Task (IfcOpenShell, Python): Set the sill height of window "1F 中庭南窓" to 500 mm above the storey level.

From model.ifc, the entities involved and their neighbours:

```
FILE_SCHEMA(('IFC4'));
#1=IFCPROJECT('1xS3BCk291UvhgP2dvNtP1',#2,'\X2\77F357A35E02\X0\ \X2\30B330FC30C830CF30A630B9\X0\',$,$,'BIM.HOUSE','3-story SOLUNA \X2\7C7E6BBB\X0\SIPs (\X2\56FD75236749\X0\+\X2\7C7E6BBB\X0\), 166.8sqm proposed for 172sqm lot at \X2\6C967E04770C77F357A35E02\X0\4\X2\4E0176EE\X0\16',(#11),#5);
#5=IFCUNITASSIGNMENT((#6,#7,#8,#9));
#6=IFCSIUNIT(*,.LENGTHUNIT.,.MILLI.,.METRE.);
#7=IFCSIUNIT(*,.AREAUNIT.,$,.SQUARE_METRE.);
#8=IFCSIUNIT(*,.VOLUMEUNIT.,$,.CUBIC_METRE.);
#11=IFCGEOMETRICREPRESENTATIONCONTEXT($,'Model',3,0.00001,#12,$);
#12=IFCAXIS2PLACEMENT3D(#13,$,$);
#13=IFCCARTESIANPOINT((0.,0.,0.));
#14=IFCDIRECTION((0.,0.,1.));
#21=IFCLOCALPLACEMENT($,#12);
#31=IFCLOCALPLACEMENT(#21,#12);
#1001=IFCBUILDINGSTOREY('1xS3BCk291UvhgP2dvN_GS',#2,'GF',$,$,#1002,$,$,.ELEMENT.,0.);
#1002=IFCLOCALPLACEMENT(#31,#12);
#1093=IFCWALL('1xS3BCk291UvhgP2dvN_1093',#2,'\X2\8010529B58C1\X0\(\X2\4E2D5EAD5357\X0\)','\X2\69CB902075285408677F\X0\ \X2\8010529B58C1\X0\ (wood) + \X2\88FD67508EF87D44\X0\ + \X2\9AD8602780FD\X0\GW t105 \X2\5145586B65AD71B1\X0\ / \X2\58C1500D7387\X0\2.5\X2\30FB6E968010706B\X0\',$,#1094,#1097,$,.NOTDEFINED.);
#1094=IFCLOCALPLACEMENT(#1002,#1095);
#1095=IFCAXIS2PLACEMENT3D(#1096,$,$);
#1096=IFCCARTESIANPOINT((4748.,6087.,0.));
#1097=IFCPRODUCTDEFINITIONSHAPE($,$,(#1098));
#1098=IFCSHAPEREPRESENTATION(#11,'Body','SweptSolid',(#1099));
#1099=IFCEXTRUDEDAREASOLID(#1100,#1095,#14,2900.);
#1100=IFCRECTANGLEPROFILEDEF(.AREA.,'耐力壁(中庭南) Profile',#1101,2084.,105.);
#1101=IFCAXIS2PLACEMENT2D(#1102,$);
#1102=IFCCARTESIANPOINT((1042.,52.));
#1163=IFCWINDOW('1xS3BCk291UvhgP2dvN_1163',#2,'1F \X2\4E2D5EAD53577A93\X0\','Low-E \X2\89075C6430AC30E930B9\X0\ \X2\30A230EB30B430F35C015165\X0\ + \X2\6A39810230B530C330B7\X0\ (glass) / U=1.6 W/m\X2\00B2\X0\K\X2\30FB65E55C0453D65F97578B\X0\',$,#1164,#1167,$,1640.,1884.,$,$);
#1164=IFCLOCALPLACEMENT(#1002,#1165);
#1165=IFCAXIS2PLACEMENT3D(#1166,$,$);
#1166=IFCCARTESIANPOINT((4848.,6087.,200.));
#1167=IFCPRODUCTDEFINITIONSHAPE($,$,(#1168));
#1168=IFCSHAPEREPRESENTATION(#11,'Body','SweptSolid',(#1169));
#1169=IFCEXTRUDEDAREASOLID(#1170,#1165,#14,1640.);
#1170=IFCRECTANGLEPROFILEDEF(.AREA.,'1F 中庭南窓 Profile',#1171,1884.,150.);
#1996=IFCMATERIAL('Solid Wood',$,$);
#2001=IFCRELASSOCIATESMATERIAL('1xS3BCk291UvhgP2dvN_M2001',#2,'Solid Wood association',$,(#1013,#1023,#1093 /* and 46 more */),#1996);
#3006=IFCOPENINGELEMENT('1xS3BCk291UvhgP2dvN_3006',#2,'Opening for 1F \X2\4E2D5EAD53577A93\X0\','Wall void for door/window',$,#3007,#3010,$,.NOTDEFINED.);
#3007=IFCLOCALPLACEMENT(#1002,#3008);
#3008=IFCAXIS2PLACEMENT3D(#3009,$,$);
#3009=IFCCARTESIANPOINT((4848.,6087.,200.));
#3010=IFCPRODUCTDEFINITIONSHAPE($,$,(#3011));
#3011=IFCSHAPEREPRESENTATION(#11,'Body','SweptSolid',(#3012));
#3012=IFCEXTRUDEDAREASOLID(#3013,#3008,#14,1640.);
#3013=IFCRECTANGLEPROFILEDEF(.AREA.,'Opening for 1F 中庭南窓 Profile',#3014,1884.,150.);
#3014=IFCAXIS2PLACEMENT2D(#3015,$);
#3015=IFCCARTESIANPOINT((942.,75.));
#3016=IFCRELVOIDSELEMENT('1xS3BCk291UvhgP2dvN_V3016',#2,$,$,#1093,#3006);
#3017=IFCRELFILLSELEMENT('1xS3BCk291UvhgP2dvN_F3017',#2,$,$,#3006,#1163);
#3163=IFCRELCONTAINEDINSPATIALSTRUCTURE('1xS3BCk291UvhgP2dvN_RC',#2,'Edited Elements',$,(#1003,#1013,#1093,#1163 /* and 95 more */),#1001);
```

```python
import numpy as np
import ifcopenshell
import ifcopenshell.api.geometry
import ifcopenshell.geom
import ifcopenshell.util.element
import ifcopenshell.util.placement
import ifcopenshell.util.shape
import ifcopenshell.util.unit

model = ifcopenshell.open("model.ifc")
unit_scale = ifcopenshell.util.unit.calculate_unit_scale(model)

window = model.by_guid("1xS3BCk291UvhgP2dvN_1163")
opening = window.FillsVoids[0].RelatingOpeningElement
storey = ifcopenshell.util.element.get_container(window, ifc_class="IfcBuildingStorey")
level = ifcopenshell.util.placement.get_local_placement(storey.ObjectPlacement)[2, 3]

# The opening's origin need not be at the sill, so measure its lowest point.
shape = ifcopenshell.geom.create_shape(ifcopenshell.geom.settings(), opening)
bottom = ifcopenshell.util.shape.get_shape_bottom_elevation(shape, shape.geometry) / unit_scale
dz = level + 0.5 / unit_scale - bottom

shift = np.array([0.0, 0.0, dz])
# The window is not placed relative to its opening, so move both.
for product in (opening, window):
    matrix = ifcopenshell.util.placement.get_local_placement(product.ObjectPlacement)
    matrix[:3, 3] += shift
    ifcopenshell.api.geometry.edit_object_placement(model, product=product, matrix=matrix, is_si=False)

print(f"moved by {dz * unit_scale:+.3f} m")

model.write("model_edited.ifc")
```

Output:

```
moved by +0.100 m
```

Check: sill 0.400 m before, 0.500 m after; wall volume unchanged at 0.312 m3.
